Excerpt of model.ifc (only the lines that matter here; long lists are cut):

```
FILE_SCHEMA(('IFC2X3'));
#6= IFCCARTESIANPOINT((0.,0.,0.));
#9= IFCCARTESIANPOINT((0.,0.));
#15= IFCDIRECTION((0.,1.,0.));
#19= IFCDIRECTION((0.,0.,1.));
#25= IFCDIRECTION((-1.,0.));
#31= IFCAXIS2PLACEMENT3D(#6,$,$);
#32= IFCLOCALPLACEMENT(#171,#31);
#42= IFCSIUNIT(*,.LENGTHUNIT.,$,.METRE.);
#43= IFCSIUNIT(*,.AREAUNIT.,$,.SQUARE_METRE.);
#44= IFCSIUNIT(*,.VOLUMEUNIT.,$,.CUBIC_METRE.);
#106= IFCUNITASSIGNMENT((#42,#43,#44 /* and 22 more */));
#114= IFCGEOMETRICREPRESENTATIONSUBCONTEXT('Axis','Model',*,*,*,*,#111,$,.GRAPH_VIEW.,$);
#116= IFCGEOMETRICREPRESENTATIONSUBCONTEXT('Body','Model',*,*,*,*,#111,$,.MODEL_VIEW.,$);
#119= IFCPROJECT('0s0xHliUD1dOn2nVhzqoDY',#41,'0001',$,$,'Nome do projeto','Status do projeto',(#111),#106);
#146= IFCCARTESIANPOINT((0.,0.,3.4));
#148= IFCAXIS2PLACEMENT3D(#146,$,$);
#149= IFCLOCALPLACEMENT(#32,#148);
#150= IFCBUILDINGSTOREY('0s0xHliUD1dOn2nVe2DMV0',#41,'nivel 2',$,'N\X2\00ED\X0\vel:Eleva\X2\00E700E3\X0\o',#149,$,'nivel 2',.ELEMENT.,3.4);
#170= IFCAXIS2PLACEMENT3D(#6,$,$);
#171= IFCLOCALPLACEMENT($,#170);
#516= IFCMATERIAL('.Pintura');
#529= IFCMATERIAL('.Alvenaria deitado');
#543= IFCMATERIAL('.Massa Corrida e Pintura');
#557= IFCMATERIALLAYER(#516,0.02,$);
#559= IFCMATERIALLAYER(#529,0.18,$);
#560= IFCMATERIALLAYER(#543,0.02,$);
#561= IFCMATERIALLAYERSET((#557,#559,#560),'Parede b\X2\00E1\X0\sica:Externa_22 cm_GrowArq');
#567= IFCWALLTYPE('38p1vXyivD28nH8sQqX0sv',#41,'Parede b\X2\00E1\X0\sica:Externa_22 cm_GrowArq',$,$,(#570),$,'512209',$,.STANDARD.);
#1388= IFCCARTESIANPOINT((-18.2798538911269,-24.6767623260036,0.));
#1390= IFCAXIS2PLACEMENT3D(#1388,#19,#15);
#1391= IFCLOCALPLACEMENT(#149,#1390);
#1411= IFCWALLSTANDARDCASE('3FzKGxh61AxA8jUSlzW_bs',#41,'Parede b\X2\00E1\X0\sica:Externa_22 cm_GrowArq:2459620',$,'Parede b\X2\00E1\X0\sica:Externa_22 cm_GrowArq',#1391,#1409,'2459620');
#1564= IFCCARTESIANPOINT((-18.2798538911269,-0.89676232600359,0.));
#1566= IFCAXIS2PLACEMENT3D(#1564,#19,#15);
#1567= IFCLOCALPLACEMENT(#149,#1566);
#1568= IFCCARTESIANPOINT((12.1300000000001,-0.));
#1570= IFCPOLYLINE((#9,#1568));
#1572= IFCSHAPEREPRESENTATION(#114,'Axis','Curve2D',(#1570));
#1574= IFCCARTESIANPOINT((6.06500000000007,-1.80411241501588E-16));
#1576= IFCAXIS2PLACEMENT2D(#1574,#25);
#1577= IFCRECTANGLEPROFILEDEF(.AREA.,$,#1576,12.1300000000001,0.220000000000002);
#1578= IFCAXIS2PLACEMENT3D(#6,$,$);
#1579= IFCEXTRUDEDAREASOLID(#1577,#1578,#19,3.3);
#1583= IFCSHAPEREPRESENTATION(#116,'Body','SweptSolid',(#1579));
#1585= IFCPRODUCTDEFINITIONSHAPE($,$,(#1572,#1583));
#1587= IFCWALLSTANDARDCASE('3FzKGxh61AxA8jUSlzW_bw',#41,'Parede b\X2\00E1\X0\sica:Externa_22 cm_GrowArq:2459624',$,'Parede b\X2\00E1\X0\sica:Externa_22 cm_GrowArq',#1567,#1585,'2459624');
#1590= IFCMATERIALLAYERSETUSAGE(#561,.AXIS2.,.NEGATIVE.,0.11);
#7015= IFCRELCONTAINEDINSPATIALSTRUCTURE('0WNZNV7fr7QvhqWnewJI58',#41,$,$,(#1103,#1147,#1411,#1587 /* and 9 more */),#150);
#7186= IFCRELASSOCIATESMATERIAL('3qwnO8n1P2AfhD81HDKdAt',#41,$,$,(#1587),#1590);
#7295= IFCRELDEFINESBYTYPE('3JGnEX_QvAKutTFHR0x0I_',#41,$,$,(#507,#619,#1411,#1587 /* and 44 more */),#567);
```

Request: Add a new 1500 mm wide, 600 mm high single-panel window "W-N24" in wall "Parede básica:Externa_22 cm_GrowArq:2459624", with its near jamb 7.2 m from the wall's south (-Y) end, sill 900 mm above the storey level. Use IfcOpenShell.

```python
import numpy as np
import ifcopenshell
import ifcopenshell.api.feature
import ifcopenshell.api.geometry
import ifcopenshell.api.root
import ifcopenshell.api.spatial
import ifcopenshell.api.type
import ifcopenshell.geom
import ifcopenshell.util.element
import ifcopenshell.util.placement
import ifcopenshell.util.representation
import ifcopenshell.util.shape
import ifcopenshell.util.unit

model = ifcopenshell.open("model.ifc")
unit_scale = ifcopenshell.util.unit.calculate_unit_scale(model)
settings = ifcopenshell.geom.settings()


def volume(element):
    """Net volume in cubic metres, openings subtracted."""
    shape = ifcopenshell.geom.create_shape(settings, element)
    return ifcopenshell.util.shape.get_volume(shape.geometry)


wall = model.by_id(1587)
storey = ifcopenshell.util.element.get_container(wall, ifc_class="IfcBuildingStorey")
context = ifcopenshell.util.representation.get_context(model, "Model", "Body", "MODEL_VIEW")
before = volume(wall)

width, height, from_end, sill = 1.5, 0.6, 7.2, 0.9  # metres

# The wall runs along its own X axis, and the end named is its -X end.
wall_shape = ifcopenshell.geom.create_shape(settings, wall)
x, y, z = ifcopenshell.util.shape.get_vertices(wall_shape.geometry).T
start = x.min() + from_end
face, thickness = float(y.min()), float(y.max() - y.min())
wall_matrix = ifcopenshell.util.placement.get_local_placement(wall.ObjectPlacement)
level = ifcopenshell.util.placement.get_local_placement(storey.ObjectPlacement)[2, 3]


def in_wall(x, y):
    """Placement at x, y metres in the wall's axes, at sill height."""
    matrix = wall_matrix.copy()
    matrix[:, 3] = wall_matrix @ np.array([x / unit_scale, y / unit_scale, 0.0, 1.0])
    matrix[2, 3] = level + sill / unit_scale
    return matrix


# Opening: a box that overshoots both wall faces by 50 mm.
opening = ifcopenshell.api.root.create_entity(model, ifc_class="IfcOpeningElement")
box = ifcopenshell.api.geometry.add_wall_representation(
    model, context=context, length=width, height=height, thickness=thickness + 0.1
)
ifcopenshell.api.geometry.assign_representation(model, product=opening, representation=box)
ifcopenshell.api.geometry.edit_object_placement(model, product=opening, matrix=in_wall(start, face - 0.05), is_si=False)
ifcopenshell.api.feature.add_feature(model, feature=opening, element=wall)

window = ifcopenshell.api.root.create_entity(model, ifc_class="IfcWindow", name="W-N24")
window.OverallWidth, window.OverallHeight = width / unit_scale, height / unit_scale
body = ifcopenshell.api.geometry.add_window_representation(
    model,
    context=context,
    overall_width=window.OverallWidth,
    overall_height=window.OverallHeight,
    partition_type="SINGLE_PANEL",
)
ifcopenshell.api.geometry.assign_representation(model, product=window, representation=body)
ifcopenshell.api.spatial.assign_container(model, products=[window], relating_structure=storey)
fills = ifcopenshell.api.feature.add_filling(model, opening=opening, element=window)
fills.OwnerHistory = window.OwnerHistory  # required in IFC2X3

# IFC2X3 keeps the operation on the window style.
style = ifcopenshell.api.root.create_entity(model, ifc_class="IfcWindowStyle", name="W-N24")
style.OperationType, style.ConstructionType = "SINGLE_PANEL", "NOTDEFINED"
style.ParameterTakesPrecedence = style.Sizeable = False
ifcopenshell.api.type.assign_type(model, related_objects=[window], relating_type=style)

# Centre the window in the wall's thickness.
ifcopenshell.api.geometry.edit_object_placement(model, product=window, matrix=in_wall(start, face), is_si=False)
window_shape = ifcopenshell.geom.create_shape(settings, window)
depth = ifcopenshell.util.shape.get_vertices(window_shape.geometry)[:, 1]
offset = face + thickness / 2 - (depth.min() + depth.max()) / 2
ifcopenshell.api.geometry.edit_object_placement(model, product=window, matrix=in_wall(start, offset), is_si=False)

after = volume(wall)

print(f"wall volume {before:.3f} -> {after:.3f} m3")

model.write("model_rev.ifc")
```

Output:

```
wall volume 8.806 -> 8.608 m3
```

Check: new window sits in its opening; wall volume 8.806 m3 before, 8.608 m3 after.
